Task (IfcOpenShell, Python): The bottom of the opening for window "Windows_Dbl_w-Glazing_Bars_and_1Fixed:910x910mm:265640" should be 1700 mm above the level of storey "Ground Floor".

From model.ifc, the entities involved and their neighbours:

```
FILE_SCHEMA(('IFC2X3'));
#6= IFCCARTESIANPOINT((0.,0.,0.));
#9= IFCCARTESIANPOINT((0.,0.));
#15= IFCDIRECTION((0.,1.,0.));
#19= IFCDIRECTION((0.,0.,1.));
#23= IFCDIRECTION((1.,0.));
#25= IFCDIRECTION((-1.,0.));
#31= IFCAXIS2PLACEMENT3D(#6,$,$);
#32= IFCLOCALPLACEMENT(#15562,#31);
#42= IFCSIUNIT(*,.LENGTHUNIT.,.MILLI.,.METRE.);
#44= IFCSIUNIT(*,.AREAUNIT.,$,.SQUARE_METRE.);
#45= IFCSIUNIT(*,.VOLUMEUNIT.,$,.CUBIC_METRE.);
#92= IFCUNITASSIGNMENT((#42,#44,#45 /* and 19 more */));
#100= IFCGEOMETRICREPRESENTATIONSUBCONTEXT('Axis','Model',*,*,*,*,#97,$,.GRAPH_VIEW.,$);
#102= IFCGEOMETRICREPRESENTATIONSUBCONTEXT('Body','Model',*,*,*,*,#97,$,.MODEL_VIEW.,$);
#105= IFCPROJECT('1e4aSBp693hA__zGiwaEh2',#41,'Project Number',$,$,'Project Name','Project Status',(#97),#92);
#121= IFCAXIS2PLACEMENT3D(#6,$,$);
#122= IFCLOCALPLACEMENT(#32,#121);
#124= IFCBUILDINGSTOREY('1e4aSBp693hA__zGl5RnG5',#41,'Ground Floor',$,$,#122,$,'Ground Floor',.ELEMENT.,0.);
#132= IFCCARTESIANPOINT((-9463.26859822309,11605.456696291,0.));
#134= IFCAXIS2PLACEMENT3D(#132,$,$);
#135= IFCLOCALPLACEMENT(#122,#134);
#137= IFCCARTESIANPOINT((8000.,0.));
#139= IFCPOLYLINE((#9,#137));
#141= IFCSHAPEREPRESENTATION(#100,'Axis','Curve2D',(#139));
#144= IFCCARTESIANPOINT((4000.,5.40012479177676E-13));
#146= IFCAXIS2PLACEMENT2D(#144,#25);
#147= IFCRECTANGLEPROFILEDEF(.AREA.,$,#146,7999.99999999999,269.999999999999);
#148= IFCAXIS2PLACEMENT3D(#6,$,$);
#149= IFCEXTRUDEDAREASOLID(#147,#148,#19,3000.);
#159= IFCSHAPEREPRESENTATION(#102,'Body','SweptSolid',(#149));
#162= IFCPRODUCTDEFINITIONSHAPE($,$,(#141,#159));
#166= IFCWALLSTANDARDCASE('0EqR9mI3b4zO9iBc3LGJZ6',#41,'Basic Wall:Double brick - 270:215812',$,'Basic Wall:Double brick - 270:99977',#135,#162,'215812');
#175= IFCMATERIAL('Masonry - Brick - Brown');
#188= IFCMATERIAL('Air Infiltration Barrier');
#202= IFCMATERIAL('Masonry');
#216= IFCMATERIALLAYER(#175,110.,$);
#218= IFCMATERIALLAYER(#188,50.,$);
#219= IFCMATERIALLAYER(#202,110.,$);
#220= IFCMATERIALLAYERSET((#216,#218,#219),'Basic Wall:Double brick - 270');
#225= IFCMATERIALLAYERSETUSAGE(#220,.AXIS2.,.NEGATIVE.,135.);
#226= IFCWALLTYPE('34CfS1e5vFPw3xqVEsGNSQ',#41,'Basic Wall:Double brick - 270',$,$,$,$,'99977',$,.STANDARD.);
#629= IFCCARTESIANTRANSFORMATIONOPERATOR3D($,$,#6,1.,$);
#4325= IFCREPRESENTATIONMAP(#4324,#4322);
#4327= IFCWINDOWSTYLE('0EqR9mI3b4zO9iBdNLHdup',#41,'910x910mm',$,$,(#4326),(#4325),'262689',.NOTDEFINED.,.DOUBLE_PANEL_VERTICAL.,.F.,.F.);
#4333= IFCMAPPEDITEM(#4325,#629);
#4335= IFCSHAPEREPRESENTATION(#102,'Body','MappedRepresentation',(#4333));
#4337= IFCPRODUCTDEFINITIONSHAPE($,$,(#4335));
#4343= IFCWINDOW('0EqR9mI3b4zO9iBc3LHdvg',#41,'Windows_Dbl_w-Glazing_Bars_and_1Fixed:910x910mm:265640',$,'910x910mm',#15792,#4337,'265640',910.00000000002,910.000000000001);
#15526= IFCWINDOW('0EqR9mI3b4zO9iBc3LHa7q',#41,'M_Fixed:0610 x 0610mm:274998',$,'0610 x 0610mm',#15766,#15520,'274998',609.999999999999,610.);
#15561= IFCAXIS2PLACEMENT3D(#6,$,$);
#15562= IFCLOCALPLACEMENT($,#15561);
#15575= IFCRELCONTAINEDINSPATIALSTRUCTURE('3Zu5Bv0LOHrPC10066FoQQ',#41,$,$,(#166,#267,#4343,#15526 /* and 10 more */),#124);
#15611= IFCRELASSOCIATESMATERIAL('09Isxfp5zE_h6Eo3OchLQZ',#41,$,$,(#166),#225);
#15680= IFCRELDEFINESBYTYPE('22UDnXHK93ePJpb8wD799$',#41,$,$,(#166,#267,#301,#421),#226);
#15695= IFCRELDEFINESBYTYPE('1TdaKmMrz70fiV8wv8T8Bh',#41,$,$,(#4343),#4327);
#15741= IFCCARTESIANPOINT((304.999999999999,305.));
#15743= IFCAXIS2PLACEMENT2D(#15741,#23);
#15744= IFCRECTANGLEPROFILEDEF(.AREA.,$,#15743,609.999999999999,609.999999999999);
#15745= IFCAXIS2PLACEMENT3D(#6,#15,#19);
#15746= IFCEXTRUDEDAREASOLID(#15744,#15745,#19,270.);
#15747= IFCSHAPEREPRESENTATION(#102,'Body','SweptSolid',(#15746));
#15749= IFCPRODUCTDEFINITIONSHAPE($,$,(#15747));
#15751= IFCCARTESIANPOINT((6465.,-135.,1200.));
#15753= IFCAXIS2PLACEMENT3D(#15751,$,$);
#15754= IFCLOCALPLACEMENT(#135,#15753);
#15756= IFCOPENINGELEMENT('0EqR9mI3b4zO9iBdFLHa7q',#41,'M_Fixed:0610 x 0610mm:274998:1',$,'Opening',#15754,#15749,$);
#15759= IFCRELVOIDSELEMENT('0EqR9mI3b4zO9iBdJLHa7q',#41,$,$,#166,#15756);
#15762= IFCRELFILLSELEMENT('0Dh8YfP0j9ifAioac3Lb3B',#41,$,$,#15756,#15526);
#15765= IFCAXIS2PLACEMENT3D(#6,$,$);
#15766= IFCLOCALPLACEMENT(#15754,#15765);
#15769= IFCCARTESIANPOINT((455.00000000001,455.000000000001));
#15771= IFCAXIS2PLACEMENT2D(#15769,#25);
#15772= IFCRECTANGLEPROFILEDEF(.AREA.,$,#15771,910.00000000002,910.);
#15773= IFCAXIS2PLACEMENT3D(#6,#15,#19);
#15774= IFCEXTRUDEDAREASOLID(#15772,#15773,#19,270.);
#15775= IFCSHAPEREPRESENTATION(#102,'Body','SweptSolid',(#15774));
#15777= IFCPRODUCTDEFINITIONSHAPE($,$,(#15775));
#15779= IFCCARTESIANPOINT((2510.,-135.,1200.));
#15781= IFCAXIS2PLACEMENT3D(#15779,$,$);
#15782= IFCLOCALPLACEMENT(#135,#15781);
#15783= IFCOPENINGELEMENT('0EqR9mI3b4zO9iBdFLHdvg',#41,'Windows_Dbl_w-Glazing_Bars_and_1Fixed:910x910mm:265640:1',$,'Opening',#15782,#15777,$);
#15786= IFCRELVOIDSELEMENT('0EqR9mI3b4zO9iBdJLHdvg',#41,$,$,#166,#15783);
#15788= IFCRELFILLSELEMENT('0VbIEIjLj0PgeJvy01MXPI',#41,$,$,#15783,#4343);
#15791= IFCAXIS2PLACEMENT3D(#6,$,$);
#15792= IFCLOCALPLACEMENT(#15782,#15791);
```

```python
import numpy as np
import ifcopenshell
import ifcopenshell.api.geometry
import ifcopenshell.geom
import ifcopenshell.util.element
import ifcopenshell.util.placement
import ifcopenshell.util.shape
import ifcopenshell.util.unit

model = ifcopenshell.open("model.ifc")
unit_scale = ifcopenshell.util.unit.calculate_unit_scale(model)

window = model.by_guid("0EqR9mI3b4zO9iBc3LHdvg")
opening = window.FillsVoids[0].RelatingOpeningElement
storey = ifcopenshell.util.element.get_container(window, ifc_class="IfcBuildingStorey")
level = ifcopenshell.util.placement.get_local_placement(storey.ObjectPlacement)[2, 3]

# The opening's origin need not be at the sill, so measure its lowest point.
shape = ifcopenshell.geom.create_shape(ifcopenshell.geom.settings(), opening)
bottom = ifcopenshell.util.shape.get_shape_bottom_elevation(shape, shape.geometry) / unit_scale
dz = level + 1.7 / unit_scale - bottom

shift = np.array([0.0, 0.0, dz])
# The window is placed relative to its opening, so it follows when the opening moves.
matrix = ifcopenshell.util.placement.get_local_placement(opening.ObjectPlacement)
matrix[:3, 3] += shift
ifcopenshell.api.geometry.edit_object_placement(
    model, product=opening, matrix=matrix, is_si=False, should_transform_children=True
)

print(f"moved by {dz * unit_scale:+.3f} m")

model.write("model_updated.ifc")
```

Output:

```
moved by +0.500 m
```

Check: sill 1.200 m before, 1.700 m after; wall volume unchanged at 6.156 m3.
